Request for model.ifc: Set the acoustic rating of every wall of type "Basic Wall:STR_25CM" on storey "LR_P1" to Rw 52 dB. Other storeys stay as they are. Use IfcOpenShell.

First a look at what the model holds.

```python
import ifcopenshell
import ifcopenshell.util.element

model = ifcopenshell.open("model.ifc")
print(model.schema)
storey = next(s for s in model.by_type("IfcBuildingStorey") if s.Name == "LR_P1")
walls = [e for e in ifcopenshell.util.element.get_decomposition(storey) if e.is_a("IfcWall")]
seen = {}
for e in walls:
    element_type = ifcopenshell.util.element.get_type(e)
    key = (element_type.Name if element_type != e and element_type else None, ifcopenshell.util.element.get_pset(e, "Pset_WallCommon", "AcousticRating"))
    seen[key] = seen.get(key, 0) + 1
for (name, value), count in sorted(seen.items(), key=str):
    print(count, "x", name, "|", value)
```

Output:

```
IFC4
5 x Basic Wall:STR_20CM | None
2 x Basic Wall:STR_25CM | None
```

```python
import ifcopenshell
import ifcopenshell.api.pset
import ifcopenshell.util.element

model = ifcopenshell.open("model.ifc")

storey = next(s for s in model.by_type("IfcBuildingStorey") if s.Name == "LR_P1")
walls = [e for e in ifcopenshell.util.element.get_decomposition(storey) if e.is_a("IfcWall")]

count = 0
for e in walls:
    element_type = ifcopenshell.util.element.get_type(e)
    if element_type in (None, e) or element_type.Name != "Basic Wall:STR_25CM":
        continue
    # add_pset returns the element's existing set when there is one.
    pset = ifcopenshell.api.pset.add_pset(model, product=e, name="Pset_WallCommon")
    ifcopenshell.api.pset.edit_pset(model, pset=pset, properties={"AcousticRating": "Rw 52 dB"})
    count += 1

print(count, "walls updated")

model.write("model_updated.ifc")
```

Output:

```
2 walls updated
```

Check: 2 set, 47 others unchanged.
